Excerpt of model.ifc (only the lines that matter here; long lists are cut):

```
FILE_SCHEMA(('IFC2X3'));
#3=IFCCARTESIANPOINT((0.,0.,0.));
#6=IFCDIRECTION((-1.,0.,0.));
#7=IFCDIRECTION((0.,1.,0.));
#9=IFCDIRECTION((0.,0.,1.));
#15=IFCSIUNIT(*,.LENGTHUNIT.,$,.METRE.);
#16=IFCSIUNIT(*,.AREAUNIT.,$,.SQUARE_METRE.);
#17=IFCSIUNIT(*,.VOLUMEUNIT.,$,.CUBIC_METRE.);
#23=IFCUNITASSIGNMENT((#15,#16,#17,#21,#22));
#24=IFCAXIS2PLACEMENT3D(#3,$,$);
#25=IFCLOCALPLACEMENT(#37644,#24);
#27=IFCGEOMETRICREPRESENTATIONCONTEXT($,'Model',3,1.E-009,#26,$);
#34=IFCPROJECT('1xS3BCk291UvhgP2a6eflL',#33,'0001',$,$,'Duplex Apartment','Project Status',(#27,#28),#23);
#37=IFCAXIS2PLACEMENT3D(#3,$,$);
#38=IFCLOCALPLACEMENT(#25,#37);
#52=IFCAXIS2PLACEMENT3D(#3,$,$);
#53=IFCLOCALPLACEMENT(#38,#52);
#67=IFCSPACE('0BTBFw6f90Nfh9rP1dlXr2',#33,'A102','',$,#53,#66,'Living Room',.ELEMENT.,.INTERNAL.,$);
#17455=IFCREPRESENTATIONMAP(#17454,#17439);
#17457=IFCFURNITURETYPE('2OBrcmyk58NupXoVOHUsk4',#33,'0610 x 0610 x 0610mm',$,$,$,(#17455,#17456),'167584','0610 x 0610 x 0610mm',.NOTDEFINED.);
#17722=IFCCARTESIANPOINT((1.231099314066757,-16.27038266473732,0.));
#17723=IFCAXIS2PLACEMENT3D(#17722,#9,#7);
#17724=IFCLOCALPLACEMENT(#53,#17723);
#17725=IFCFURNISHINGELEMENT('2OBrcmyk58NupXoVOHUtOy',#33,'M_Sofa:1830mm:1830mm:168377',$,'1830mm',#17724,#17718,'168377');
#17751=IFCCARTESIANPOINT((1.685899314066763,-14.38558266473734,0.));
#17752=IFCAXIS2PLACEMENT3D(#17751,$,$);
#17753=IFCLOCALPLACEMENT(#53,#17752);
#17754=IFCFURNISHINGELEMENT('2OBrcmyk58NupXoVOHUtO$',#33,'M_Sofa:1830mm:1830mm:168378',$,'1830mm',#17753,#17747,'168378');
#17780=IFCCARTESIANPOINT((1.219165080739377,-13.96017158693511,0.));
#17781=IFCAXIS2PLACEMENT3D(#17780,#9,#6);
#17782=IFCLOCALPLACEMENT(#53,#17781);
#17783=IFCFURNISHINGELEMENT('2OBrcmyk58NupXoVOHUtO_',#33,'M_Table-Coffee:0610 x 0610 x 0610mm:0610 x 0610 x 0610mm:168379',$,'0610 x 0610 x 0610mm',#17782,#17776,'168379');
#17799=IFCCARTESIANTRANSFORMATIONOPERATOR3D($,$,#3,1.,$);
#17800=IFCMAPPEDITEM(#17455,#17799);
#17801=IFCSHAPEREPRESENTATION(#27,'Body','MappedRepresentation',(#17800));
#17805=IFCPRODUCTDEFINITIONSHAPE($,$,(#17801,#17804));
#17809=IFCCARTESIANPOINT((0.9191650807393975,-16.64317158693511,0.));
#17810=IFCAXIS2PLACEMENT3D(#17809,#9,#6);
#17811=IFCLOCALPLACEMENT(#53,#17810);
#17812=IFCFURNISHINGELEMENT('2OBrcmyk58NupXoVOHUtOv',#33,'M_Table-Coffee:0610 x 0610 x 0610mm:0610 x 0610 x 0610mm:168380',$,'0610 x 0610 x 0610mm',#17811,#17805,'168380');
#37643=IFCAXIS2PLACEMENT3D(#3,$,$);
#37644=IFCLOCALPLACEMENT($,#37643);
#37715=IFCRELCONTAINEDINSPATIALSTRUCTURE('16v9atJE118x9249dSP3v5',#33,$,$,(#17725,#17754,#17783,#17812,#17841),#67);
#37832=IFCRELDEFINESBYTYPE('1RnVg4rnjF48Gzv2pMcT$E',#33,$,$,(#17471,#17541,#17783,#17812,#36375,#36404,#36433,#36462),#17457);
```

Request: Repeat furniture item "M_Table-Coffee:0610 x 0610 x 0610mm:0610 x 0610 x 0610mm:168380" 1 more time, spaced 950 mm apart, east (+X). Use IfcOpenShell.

```python
import numpy as np
import ifcopenshell
import ifcopenshell.api.geometry
import ifcopenshell.api.root
import ifcopenshell.util.element
import ifcopenshell.util.placement
import ifcopenshell.util.unit

model = ifcopenshell.open("model.ifc")
unit_scale = ifcopenshell.util.unit.calculate_unit_scale(model)


def reuse_history(source, copy):
    """copy_class also copies each property set's owner history, people and application; keep the originals."""
    for rel in copy.IsDefinedBy:
        if rel.is_a("IfcRelDefinesByProperties") and (history := rel.RelatingPropertyDefinition.OwnerHistory):
            rel.RelatingPropertyDefinition.OwnerHistory = source.OwnerHistory
            ifcopenshell.util.element.remove_deep2(model, history)


source = model.by_id(17812)
base = ifcopenshell.util.placement.get_local_placement(source.ObjectPlacement)
step = np.array([1.0, 0.0, 0.0]) * 0.95 / unit_scale

for i in range(1, 2):
    copy = ifcopenshell.api.root.copy_class(model, product=source)
    copy.Representation = ifcopenshell.util.element.copy_deep(
        model, source.Representation, exclude=["IfcGeometricRepresentationContext", "IfcRepresentationMap"]
    )
    copy.Name = "M_Table-Coffee:0610 x 0610 x 0610mm:0610 x 0610 x 0610mm"
    copy.Tag = None
    reuse_history(source, copy)
    matrix = base.copy()
    matrix[:3, 3] += i * step
    print("added at", matrix[:3, 3].round(3) + 0.0)
    ifcopenshell.api.geometry.edit_object_placement(model, product=copy, matrix=matrix, is_si=False)

model.write("model_v2.ifc")
```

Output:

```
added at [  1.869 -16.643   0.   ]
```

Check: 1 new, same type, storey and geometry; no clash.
